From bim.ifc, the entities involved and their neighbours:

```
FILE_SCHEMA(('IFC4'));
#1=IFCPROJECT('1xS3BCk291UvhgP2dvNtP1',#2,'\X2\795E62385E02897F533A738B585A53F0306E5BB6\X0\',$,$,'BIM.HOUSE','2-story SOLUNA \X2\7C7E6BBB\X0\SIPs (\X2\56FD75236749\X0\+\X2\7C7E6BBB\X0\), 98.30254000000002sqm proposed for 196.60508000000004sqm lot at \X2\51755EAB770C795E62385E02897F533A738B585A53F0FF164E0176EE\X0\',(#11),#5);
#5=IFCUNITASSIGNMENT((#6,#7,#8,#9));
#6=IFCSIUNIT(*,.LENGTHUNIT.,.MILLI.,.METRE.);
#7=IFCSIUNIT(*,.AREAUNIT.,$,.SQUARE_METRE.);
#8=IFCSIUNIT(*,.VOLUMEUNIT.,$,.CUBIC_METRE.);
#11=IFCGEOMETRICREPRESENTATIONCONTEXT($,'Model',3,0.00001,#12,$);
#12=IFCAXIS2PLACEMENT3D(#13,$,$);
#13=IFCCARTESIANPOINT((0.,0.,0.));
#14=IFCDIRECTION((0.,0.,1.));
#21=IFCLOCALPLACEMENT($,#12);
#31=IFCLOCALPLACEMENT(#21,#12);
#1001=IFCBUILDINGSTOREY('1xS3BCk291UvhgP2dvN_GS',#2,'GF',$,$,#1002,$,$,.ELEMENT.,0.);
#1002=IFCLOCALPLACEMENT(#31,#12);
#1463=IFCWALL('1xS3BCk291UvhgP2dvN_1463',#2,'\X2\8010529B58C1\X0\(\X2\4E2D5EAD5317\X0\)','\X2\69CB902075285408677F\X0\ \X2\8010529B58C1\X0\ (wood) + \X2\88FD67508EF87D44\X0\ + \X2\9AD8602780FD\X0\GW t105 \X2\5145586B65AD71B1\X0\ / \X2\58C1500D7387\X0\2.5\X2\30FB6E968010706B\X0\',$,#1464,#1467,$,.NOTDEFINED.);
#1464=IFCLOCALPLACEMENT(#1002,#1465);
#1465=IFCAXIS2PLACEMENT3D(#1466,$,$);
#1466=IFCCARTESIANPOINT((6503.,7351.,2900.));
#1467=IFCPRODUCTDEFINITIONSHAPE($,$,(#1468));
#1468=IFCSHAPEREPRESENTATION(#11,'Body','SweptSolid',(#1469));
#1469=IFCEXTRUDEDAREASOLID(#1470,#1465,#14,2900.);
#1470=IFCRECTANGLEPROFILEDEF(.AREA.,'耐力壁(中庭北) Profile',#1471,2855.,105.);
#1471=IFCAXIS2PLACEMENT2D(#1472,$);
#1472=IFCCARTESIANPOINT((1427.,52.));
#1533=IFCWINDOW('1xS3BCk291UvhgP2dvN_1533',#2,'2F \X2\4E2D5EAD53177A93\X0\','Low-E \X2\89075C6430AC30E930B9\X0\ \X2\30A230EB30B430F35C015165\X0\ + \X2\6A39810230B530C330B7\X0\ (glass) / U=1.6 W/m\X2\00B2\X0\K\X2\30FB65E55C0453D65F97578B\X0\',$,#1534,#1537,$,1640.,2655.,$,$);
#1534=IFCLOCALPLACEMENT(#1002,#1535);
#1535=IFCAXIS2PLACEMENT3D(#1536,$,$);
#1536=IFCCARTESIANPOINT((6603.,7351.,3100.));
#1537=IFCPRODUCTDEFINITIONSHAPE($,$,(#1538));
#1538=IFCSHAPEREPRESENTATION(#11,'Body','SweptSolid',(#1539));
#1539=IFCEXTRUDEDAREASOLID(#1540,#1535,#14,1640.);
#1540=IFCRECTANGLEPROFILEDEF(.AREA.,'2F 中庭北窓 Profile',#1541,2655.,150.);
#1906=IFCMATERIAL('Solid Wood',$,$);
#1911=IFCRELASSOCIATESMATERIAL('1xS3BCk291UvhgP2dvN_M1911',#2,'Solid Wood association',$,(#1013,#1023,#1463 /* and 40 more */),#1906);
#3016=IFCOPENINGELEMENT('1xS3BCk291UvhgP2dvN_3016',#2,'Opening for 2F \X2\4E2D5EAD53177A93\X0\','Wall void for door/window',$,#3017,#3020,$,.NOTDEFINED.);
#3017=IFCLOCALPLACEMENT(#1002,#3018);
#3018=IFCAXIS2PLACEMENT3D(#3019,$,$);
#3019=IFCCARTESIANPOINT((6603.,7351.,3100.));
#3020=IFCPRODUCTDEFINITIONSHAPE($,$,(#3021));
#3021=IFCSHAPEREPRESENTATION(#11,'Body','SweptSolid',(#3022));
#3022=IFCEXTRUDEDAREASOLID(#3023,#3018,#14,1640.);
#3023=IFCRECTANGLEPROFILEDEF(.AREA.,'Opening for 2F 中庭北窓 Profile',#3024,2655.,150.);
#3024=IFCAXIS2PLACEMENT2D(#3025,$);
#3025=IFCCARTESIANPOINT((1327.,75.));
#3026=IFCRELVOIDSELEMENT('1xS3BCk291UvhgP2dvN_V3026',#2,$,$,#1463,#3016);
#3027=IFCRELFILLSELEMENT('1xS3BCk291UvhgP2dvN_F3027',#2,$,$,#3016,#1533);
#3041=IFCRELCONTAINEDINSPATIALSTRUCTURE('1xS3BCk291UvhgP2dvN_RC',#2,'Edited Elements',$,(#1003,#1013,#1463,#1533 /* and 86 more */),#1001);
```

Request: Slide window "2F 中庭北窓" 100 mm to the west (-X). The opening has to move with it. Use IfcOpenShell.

```python
import ifcopenshell
import ifcopenshell.api.geometry
import ifcopenshell.util.placement

model = ifcopenshell.open("bim.ifc")

window = model.by_guid("1xS3BCk291UvhgP2dvN_1533")
opening = window.FillsVoids[0].RelatingOpeningElement
wall = opening.VoidsElements[0].RelatingBuildingElement

wall_matrix = ifcopenshell.util.placement.get_local_placement(wall.ObjectPlacement)
shift = wall_matrix[:3, 0] * -100.0
before = ifcopenshell.util.placement.get_local_placement(window.ObjectPlacement)[:3, 3].copy()

# The window is not placed relative to its opening, so move both.
for product in (opening, window):
    matrix = ifcopenshell.util.placement.get_local_placement(product.ObjectPlacement)
    matrix[:3, 3] += shift
    ifcopenshell.api.geometry.edit_object_placement(model, product=product, matrix=matrix, is_si=False)

after = ifcopenshell.util.placement.get_local_placement(window.ObjectPlacement)[:3, 3]
print("window moved by", (after - before).round(3) + 0.0)

model.write("bim_edited.ifc")
```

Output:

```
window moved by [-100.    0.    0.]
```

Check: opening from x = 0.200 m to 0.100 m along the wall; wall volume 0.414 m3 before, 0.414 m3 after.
